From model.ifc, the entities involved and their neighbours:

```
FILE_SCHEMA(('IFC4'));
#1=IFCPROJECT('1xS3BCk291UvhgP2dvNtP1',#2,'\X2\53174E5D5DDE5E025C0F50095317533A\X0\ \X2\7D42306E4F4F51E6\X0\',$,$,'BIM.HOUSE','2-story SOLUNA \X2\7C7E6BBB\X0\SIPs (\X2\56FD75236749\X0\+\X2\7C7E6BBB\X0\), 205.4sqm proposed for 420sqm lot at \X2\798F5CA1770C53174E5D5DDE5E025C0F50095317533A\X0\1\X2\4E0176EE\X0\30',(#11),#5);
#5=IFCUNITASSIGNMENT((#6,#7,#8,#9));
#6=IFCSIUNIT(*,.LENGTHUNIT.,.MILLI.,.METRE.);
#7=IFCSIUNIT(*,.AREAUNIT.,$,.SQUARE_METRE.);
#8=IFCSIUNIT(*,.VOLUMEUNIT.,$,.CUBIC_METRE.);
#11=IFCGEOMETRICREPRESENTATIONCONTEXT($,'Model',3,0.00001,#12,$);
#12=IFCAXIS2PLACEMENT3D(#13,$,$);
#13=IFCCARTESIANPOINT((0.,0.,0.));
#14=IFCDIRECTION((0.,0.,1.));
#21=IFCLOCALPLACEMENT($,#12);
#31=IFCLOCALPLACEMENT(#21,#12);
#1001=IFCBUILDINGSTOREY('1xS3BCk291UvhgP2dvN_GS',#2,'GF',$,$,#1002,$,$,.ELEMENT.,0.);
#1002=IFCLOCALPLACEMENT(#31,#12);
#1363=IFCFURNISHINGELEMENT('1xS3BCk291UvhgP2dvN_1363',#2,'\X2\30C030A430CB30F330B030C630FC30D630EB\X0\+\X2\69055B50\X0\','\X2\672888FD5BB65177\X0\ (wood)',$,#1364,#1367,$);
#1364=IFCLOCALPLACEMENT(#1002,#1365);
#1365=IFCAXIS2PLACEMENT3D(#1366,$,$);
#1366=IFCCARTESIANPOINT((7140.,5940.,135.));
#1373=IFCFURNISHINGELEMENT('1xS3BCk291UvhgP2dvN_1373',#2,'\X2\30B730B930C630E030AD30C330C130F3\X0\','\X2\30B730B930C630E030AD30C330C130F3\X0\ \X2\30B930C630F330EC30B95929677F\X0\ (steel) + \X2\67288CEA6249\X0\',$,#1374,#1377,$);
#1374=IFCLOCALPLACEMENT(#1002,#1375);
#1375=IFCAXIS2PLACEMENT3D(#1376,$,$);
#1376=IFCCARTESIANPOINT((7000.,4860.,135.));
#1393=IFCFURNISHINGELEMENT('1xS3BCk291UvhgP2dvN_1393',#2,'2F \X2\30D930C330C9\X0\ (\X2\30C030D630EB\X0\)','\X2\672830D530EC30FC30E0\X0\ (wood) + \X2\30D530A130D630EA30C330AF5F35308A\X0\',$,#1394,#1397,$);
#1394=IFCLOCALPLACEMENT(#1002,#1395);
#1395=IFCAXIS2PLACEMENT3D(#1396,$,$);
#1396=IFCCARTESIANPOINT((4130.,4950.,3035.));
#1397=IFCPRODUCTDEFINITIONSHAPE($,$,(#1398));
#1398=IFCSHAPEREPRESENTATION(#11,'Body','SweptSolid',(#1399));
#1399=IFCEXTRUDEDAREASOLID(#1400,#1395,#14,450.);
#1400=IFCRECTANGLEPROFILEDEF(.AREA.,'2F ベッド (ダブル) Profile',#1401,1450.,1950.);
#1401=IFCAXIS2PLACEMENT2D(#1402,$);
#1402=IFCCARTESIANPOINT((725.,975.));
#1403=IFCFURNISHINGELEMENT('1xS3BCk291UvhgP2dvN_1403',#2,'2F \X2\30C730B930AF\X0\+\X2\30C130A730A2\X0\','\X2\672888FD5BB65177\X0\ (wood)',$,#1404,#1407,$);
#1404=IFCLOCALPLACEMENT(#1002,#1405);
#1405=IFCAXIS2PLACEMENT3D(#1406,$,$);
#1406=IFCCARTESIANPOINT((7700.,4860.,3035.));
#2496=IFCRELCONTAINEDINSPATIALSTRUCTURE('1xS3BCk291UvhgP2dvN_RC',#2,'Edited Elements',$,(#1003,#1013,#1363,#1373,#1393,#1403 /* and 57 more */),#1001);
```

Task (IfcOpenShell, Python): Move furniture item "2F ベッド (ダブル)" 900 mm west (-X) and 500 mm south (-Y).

```python
import ifcopenshell
import ifcopenshell.api.geometry
import ifcopenshell.util.placement

model = ifcopenshell.open("model.ifc")

item = model.by_guid("1xS3BCk291UvhgP2dvN_1393")
matrix = ifcopenshell.util.placement.get_local_placement(item.ObjectPlacement)
matrix[0, 3] -= 900.0
matrix[1, 3] -= 500.0
ifcopenshell.api.geometry.edit_object_placement(model, product=item, matrix=matrix, is_si=False)

print(ifcopenshell.util.placement.get_local_placement(item.ObjectPlacement).round(3) + 0.0)

model.write("model_rev.ifc")
```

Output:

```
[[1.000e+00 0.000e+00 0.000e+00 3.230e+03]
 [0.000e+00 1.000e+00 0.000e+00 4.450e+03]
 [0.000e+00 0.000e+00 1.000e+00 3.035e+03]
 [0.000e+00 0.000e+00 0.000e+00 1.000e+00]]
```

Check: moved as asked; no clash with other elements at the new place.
